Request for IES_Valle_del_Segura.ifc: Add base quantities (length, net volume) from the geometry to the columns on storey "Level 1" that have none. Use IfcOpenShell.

First a look at what the model holds.

```python
import ifcopenshell
import ifcopenshell.util.element
import ifcopenshell.util.unit

model = ifcopenshell.open("IES_Valle_del_Segura.ifc")
print(model.schema)
for unit_type in ("LENGTHUNIT", "AREAUNIT", "VOLUMEUNIT"):
    print(unit_type, ifcopenshell.util.unit.calculate_unit_scale(model, unit_type))
storey = next(s for s in model.by_type("IfcBuildingStorey") if s.Name == "Level 1")
columns = [e for e in ifcopenshell.util.element.get_decomposition(storey) if e.is_a("IfcColumn")]
for e in sorted(columns, key=lambda e: e.id()):
    print(e.id(), e.is_a(), e.Name, list(ifcopenshell.util.element.get_psets(e, qtos_only=True)), sep=" | ")
```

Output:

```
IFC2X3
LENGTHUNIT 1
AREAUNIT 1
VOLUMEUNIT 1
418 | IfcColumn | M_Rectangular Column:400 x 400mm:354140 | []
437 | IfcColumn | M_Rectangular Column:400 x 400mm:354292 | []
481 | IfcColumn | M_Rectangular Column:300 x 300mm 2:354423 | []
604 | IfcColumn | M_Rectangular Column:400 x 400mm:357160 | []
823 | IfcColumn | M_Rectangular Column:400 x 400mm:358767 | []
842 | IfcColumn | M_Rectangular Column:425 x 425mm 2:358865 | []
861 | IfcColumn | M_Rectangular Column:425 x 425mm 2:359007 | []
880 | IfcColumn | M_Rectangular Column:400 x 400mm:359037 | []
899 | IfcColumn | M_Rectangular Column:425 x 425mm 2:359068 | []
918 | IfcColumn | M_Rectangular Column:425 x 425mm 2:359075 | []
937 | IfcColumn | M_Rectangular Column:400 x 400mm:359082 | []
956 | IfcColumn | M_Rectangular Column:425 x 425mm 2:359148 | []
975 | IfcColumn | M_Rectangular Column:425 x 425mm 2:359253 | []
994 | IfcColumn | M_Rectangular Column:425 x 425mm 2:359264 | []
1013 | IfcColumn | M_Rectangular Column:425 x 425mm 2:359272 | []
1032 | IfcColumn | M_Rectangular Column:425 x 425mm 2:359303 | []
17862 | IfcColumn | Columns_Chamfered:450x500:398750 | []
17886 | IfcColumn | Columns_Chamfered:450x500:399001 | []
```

```python
import ifcopenshell
import ifcopenshell.api.pset
import ifcopenshell.geom
import ifcopenshell.util.element
import ifcopenshell.util.shape
import ifcopenshell.util.unit

model = ifcopenshell.open("IES_Valle_del_Segura.ifc")
unit_scale = ifcopenshell.util.unit.calculate_unit_scale(model)
volume_scale = ifcopenshell.util.unit.calculate_unit_scale(model, "VOLUMEUNIT")
settings = ifcopenshell.geom.settings()

storey = next(s for s in model.by_type("IfcBuildingStorey") if s.Name == "Level 1")
columns = [e for e in ifcopenshell.util.element.get_decomposition(storey) if e.is_a("IfcColumn")]

for e in sorted(columns, key=lambda e: e.id()):
    if ifcopenshell.util.element.get_psets(e, qtos_only=True, should_inherit=False):
        continue
    # Geometry comes back in metres, in the element's own axes.
    shape = ifcopenshell.geom.create_shape(settings, e)
    values = {
        "Length": ifcopenshell.util.shape.get_z(shape.geometry) / unit_scale,
        "NetVolume": ifcopenshell.util.shape.get_volume(shape.geometry) / volume_scale,
    }
    qto = ifcopenshell.api.pset.add_qto(model, product=e, name="BaseQuantities")
    ifcopenshell.api.pset.edit_qto(model, qto=qto, properties=values)
    print(e.id(), {k: round(v, 3) for k, v in values.items()})

model.write("IES_Valle_del_Segura_rev.ifc")
```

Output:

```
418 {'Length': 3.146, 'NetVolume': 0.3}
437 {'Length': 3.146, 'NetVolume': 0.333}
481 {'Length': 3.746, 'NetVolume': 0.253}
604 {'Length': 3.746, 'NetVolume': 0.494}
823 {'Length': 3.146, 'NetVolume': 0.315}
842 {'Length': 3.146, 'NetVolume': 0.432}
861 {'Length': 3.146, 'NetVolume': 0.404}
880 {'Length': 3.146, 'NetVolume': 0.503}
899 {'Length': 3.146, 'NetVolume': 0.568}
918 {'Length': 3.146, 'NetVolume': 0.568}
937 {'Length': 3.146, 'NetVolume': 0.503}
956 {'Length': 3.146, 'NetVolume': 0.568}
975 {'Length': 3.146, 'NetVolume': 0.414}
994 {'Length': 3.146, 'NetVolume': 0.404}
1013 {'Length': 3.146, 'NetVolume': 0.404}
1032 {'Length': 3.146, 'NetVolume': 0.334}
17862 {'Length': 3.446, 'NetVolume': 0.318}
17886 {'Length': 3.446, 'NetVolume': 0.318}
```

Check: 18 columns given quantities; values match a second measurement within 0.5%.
